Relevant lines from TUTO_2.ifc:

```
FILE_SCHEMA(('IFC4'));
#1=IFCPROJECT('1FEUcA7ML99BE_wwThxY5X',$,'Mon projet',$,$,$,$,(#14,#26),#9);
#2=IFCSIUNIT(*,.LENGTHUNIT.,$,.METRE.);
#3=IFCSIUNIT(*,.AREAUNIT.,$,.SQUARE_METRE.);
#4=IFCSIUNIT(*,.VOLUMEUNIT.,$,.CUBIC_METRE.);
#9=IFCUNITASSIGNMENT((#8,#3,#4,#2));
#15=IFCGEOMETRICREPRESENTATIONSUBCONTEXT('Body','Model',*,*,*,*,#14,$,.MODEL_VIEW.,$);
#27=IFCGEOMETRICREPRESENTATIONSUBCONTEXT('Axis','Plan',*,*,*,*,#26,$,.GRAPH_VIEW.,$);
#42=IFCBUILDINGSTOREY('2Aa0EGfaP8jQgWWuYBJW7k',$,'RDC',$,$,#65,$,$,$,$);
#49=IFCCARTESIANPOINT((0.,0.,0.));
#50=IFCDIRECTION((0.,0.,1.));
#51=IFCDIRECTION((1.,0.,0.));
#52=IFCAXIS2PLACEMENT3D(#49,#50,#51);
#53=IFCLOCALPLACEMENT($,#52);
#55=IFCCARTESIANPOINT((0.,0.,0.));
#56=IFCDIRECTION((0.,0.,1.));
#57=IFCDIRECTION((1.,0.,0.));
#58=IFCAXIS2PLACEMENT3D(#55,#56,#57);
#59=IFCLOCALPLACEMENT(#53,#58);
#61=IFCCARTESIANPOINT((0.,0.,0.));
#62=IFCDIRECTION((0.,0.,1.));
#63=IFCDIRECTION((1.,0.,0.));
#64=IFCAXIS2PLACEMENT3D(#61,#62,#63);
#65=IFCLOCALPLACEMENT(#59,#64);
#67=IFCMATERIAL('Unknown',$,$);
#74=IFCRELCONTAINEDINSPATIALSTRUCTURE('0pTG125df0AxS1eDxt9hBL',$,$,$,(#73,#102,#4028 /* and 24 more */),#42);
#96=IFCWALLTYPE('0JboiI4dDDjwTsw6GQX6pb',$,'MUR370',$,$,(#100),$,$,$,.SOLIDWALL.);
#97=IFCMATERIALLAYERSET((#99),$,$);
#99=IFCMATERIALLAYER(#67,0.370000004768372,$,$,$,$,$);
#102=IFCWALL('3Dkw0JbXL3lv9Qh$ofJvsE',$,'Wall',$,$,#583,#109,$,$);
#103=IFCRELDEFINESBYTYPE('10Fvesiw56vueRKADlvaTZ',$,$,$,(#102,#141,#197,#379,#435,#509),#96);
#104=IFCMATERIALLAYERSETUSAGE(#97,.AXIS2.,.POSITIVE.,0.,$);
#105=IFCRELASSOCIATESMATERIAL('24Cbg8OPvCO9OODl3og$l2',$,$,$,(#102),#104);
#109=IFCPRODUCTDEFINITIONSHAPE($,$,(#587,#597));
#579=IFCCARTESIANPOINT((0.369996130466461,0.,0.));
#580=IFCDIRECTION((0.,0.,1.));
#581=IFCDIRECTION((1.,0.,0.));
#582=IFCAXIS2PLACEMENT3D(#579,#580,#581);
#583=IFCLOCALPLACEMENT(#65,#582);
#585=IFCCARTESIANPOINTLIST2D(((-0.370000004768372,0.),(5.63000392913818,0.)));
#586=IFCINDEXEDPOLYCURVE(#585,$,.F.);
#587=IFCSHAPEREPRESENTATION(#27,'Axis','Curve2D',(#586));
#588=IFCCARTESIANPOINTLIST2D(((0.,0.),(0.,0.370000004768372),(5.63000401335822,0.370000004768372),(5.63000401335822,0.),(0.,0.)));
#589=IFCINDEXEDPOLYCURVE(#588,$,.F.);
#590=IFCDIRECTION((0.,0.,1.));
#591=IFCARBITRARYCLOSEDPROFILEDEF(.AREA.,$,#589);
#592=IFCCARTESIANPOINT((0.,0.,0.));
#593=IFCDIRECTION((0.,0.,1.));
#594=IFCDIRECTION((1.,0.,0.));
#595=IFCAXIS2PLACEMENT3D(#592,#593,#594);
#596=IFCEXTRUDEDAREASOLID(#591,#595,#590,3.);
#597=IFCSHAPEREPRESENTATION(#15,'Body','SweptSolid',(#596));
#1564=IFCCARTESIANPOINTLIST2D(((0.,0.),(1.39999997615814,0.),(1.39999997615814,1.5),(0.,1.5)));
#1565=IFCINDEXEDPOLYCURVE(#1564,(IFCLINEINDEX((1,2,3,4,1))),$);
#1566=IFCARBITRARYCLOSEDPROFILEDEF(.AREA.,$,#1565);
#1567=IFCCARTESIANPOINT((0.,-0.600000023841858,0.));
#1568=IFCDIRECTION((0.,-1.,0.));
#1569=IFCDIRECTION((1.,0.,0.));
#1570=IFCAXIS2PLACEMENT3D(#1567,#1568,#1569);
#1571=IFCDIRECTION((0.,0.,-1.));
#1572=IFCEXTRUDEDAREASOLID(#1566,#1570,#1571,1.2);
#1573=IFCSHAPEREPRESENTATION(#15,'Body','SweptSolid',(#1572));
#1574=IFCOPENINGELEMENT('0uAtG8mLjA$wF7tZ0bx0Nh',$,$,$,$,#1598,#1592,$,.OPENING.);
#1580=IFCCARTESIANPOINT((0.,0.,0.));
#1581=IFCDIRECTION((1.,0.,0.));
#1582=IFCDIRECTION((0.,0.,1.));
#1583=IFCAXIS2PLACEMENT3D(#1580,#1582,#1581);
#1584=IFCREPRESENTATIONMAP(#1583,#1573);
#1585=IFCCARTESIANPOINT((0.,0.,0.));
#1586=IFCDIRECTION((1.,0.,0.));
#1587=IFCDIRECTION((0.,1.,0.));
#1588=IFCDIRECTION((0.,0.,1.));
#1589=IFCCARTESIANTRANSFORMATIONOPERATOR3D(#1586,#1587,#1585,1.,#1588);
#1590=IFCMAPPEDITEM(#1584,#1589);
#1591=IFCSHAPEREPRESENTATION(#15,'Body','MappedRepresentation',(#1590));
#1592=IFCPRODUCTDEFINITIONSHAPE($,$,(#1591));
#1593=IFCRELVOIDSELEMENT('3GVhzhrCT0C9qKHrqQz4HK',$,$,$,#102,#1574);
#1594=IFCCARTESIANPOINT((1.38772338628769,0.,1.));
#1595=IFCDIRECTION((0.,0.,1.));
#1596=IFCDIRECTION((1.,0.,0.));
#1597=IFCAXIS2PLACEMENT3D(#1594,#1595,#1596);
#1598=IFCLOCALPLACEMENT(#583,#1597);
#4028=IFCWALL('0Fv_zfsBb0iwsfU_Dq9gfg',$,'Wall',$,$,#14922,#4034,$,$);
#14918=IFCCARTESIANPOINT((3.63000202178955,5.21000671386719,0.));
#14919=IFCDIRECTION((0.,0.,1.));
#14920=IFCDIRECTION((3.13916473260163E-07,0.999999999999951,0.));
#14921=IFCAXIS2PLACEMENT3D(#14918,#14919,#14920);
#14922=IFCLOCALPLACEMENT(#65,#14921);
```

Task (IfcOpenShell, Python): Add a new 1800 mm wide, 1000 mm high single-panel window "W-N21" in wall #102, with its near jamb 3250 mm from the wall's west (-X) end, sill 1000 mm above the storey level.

```python
import numpy as np
import ifcopenshell
import ifcopenshell.api.feature
import ifcopenshell.api.geometry
import ifcopenshell.api.root
import ifcopenshell.api.spatial
import ifcopenshell.geom
import ifcopenshell.util.element
import ifcopenshell.util.placement
import ifcopenshell.util.representation
import ifcopenshell.util.shape
import ifcopenshell.util.unit

model = ifcopenshell.open("TUTO_2.ifc")
unit_scale = ifcopenshell.util.unit.calculate_unit_scale(model)
settings = ifcopenshell.geom.settings()


def volume(element):
    """Net volume in cubic metres, openings subtracted."""
    shape = ifcopenshell.geom.create_shape(settings, element)
    return ifcopenshell.util.shape.get_volume(shape.geometry)


wall = model.by_guid("3Dkw0JbXL3lv9Qh$ofJvsE")
storey = ifcopenshell.util.element.get_container(wall, ifc_class="IfcBuildingStorey")
context = ifcopenshell.util.representation.get_context(model, "Model", "Body", "MODEL_VIEW")
before = volume(wall)

width, height, from_end, sill = 1.8, 1, 3.25, 1  # metres

# The wall runs along its own X axis, and the end named is its -X end.
wall_shape = ifcopenshell.geom.create_shape(settings, wall)
x, y, z = ifcopenshell.util.shape.get_vertices(wall_shape.geometry).T
start = x.min() + from_end
face, thickness = float(y.min()), float(y.max() - y.min())
wall_matrix = ifcopenshell.util.placement.get_local_placement(wall.ObjectPlacement)
level = ifcopenshell.util.placement.get_local_placement(storey.ObjectPlacement)[2, 3]


def in_wall(x, y):
    """Placement at x, y metres in the wall's axes, at sill height."""
    matrix = wall_matrix.copy()
    matrix[:, 3] = wall_matrix @ np.array([x / unit_scale, y / unit_scale, 0.0, 1.0])
    matrix[2, 3] = level + sill / unit_scale
    return matrix


# Opening: a box that overshoots both wall faces by 50 mm.
opening = ifcopenshell.api.root.create_entity(model, ifc_class="IfcOpeningElement", predefined_type="OPENING")
box = ifcopenshell.api.geometry.add_wall_representation(
    model, context=context, length=width, height=height, thickness=thickness + 0.1
)
ifcopenshell.api.geometry.assign_representation(model, product=opening, representation=box)
ifcopenshell.api.geometry.edit_object_placement(model, product=opening, matrix=in_wall(start, face - 0.05), is_si=False)
ifcopenshell.api.feature.add_feature(model, feature=opening, element=wall)

window = ifcopenshell.api.root.create_entity(model, ifc_class="IfcWindow", name="W-N21", predefined_type="WINDOW")
window.OverallWidth, window.OverallHeight = width / unit_scale, height / unit_scale
window.PartitioningType = "SINGLE_PANEL"
body = ifcopenshell.api.geometry.add_window_representation(
    model,
    context=context,
    overall_width=window.OverallWidth,
    overall_height=window.OverallHeight,
    partition_type="SINGLE_PANEL",
)
ifcopenshell.api.geometry.assign_representation(model, product=window, representation=body)
ifcopenshell.api.spatial.assign_container(model, products=[window], relating_structure=storey)
ifcopenshell.api.feature.add_filling(model, opening=opening, element=window)

# Centre the window in the wall's thickness.
ifcopenshell.api.geometry.edit_object_placement(model, product=window, matrix=in_wall(start, face), is_si=False)
window_shape = ifcopenshell.geom.create_shape(settings, window)
depth = ifcopenshell.util.shape.get_vertices(window_shape.geometry)[:, 1]
offset = face + thickness / 2 - (depth.min() + depth.max()) / 2
ifcopenshell.api.geometry.edit_object_placement(model, product=window, matrix=in_wall(start, offset), is_si=False)

after = volume(wall)

print(f"wall volume {before:.3f} -> {after:.3f} m3")

model.write("TUTO_2_rev.ifc")
```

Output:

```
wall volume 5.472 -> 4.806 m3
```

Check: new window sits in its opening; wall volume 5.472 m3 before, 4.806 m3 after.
